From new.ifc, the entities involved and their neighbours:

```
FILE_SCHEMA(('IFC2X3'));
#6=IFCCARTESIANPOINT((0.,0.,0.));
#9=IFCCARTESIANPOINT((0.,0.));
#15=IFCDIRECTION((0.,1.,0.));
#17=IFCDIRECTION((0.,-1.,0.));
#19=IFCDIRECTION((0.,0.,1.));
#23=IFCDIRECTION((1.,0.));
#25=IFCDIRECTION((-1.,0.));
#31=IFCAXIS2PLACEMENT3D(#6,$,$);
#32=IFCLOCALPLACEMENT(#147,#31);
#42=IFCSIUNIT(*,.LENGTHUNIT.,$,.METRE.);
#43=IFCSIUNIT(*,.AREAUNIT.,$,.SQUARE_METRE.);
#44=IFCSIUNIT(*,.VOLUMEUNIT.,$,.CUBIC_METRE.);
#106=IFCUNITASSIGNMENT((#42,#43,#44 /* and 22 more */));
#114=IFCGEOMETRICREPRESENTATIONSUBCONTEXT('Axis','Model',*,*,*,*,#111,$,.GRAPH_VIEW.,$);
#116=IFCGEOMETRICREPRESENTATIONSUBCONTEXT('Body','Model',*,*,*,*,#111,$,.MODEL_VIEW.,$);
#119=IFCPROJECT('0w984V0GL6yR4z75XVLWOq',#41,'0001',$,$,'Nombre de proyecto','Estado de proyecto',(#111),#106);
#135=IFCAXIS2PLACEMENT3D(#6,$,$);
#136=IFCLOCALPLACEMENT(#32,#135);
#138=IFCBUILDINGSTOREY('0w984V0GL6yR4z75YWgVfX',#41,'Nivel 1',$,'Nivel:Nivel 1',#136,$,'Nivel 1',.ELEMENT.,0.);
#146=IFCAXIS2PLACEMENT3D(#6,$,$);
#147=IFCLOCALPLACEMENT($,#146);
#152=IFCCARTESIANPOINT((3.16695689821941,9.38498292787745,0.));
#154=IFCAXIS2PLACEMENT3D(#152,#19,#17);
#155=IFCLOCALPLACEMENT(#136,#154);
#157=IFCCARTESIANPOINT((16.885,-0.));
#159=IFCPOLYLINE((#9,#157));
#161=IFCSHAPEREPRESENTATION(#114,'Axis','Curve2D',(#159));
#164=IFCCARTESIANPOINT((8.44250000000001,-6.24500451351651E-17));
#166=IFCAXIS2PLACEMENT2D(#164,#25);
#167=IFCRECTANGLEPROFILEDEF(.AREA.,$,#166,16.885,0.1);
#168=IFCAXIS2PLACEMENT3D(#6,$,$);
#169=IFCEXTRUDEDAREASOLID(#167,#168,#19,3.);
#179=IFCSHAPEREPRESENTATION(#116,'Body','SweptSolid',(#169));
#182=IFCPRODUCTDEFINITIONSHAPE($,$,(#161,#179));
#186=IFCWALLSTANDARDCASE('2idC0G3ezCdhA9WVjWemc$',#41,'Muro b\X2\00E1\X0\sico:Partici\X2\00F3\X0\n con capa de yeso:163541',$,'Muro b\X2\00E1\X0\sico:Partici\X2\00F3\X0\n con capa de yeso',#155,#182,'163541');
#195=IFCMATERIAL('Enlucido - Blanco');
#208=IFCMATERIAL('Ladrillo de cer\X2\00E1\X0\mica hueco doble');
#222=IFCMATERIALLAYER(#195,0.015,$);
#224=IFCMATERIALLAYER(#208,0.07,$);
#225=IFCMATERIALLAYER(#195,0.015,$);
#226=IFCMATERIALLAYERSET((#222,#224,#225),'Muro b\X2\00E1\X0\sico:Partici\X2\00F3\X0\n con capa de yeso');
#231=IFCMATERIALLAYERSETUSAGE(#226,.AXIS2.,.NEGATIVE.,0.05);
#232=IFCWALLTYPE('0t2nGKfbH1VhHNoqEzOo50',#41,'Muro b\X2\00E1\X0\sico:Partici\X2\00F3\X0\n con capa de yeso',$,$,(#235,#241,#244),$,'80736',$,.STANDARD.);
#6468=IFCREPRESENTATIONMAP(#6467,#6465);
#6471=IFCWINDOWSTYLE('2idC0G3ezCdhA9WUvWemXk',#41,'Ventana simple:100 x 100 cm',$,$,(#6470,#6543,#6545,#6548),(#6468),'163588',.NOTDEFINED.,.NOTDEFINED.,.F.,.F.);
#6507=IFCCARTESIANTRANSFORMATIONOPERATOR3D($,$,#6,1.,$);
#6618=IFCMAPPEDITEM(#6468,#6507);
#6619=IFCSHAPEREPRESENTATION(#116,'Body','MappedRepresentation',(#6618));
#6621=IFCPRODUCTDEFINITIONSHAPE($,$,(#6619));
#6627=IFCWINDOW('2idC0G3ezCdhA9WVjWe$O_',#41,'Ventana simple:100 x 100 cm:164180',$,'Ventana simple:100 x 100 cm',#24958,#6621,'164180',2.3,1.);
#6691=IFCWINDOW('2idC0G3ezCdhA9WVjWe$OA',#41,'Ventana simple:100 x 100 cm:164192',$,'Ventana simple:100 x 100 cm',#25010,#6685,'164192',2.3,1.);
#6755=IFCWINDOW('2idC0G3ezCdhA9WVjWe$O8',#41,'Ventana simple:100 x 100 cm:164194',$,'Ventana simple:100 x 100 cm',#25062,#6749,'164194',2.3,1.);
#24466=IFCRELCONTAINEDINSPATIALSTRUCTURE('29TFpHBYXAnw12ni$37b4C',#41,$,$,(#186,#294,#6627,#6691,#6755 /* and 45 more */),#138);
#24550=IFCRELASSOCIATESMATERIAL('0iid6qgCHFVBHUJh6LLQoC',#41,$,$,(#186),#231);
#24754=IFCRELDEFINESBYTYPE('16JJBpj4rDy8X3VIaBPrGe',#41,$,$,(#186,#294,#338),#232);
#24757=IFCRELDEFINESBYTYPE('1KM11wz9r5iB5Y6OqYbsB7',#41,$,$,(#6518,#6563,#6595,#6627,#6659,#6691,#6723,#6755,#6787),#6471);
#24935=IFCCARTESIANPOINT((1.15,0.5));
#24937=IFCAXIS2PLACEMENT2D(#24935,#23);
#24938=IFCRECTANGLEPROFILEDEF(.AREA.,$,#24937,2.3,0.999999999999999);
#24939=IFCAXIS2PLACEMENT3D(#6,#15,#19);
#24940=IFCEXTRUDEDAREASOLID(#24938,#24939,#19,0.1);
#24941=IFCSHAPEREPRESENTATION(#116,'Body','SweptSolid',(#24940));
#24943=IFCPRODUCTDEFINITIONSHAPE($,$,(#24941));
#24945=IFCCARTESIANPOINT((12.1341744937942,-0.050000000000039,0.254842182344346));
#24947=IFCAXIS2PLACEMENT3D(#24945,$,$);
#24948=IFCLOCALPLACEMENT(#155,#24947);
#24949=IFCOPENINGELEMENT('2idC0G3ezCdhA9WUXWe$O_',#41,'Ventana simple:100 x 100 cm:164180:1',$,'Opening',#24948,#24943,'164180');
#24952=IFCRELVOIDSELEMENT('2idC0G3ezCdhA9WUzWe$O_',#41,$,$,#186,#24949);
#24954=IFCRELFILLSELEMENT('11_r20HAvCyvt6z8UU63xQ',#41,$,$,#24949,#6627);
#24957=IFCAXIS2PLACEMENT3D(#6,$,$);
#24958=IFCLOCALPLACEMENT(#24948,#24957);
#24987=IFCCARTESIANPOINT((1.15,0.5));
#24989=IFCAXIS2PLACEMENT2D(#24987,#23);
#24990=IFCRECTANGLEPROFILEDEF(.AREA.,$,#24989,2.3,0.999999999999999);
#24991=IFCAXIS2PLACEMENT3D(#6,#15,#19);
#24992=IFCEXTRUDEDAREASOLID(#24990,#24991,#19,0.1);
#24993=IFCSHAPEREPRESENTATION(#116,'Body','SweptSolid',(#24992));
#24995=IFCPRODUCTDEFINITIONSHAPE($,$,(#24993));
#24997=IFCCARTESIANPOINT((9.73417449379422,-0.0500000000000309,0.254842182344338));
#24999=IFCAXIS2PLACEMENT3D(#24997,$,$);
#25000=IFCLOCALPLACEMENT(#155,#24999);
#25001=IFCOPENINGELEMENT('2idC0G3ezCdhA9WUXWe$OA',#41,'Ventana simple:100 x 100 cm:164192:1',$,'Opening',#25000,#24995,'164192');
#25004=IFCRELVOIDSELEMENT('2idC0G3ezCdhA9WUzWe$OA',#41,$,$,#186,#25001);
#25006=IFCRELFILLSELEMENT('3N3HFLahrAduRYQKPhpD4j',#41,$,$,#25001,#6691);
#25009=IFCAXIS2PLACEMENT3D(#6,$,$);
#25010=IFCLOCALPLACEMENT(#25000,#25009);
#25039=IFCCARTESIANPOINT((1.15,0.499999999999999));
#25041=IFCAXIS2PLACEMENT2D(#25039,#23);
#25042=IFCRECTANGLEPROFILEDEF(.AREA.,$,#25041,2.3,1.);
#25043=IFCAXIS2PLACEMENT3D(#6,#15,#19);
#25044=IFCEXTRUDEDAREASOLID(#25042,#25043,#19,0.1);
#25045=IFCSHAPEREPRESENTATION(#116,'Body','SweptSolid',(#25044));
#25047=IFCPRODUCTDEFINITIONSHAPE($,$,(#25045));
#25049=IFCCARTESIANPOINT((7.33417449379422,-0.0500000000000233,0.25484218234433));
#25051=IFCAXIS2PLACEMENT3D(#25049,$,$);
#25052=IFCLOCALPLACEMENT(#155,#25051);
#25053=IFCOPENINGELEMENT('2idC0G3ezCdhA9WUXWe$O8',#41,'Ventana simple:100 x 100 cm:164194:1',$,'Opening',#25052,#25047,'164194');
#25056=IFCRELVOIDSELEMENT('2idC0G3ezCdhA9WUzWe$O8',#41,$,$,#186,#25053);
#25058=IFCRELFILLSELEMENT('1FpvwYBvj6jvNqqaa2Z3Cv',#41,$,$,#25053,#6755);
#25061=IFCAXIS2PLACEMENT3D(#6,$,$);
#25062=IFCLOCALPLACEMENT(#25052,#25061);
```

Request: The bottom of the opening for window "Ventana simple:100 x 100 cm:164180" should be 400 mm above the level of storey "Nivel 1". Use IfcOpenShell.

```python
import numpy as np
import ifcopenshell
import ifcopenshell.api.geometry
import ifcopenshell.geom
import ifcopenshell.util.element
import ifcopenshell.util.placement
import ifcopenshell.util.shape
import ifcopenshell.util.unit

model = ifcopenshell.open("new.ifc")
unit_scale = ifcopenshell.util.unit.calculate_unit_scale(model)

window = model.by_id(6627)
opening = window.FillsVoids[0].RelatingOpeningElement
storey = ifcopenshell.util.element.get_container(window, ifc_class="IfcBuildingStorey")
level = ifcopenshell.util.placement.get_local_placement(storey.ObjectPlacement)[2, 3]

# The opening's origin need not be at the sill, so measure its lowest point.
shape = ifcopenshell.geom.create_shape(ifcopenshell.geom.settings(), opening)
bottom = ifcopenshell.util.shape.get_shape_bottom_elevation(shape, shape.geometry) / unit_scale
dz = level + 0.4 / unit_scale - bottom

shift = np.array([0.0, 0.0, dz])
# The window is placed relative to its opening, so it follows when the opening moves.
matrix = ifcopenshell.util.placement.get_local_placement(opening.ObjectPlacement)
matrix[:3, 3] += shift
ifcopenshell.api.geometry.edit_object_placement(
    model, product=opening, matrix=matrix, is_si=False, should_transform_children=True
)

print(f"moved by {dz * unit_scale:+.3f} m")

model.write("new_rev.ifc")
```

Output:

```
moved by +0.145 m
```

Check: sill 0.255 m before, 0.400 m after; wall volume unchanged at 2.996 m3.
